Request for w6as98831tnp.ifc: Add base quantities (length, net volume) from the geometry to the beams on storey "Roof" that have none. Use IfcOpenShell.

First a look at what the model holds.

```python
import ifcopenshell
import ifcopenshell.util.element
import ifcopenshell.util.unit

model = ifcopenshell.open("w6as98831tnp.ifc")
print(model.schema)
for unit_type in ("LENGTHUNIT", "AREAUNIT", "VOLUMEUNIT"):
    print(unit_type, ifcopenshell.util.unit.calculate_unit_scale(model, unit_type))
storey = next(s for s in model.by_type("IfcBuildingStorey") if s.Name == "Roof")
beams = [e for e in ifcopenshell.util.element.get_decomposition(storey) if e.is_a("IfcBeam")]
for e in sorted(beams, key=lambda e: e.id()):
    print(e.id(), e.is_a(), e.Name, list(ifcopenshell.util.element.get_psets(e, qtos_only=True)), sep=" | ")
```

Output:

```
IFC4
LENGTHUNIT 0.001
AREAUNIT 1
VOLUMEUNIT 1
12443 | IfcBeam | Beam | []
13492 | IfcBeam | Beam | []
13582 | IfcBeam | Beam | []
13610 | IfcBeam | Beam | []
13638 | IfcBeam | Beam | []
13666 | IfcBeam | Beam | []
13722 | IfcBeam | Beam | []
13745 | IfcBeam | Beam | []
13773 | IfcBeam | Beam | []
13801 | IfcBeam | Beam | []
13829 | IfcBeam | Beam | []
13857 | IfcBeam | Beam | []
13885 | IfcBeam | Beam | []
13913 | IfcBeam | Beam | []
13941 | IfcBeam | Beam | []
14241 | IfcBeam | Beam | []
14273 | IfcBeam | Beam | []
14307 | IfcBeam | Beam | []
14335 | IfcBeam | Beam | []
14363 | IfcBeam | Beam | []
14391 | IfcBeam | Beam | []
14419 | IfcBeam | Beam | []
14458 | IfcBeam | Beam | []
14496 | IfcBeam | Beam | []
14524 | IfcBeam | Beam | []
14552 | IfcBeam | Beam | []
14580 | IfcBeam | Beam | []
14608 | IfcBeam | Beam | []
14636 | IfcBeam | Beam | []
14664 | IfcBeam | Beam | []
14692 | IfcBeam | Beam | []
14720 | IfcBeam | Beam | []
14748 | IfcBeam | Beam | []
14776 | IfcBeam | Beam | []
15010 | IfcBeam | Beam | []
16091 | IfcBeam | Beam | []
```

```python
import ifcopenshell
import ifcopenshell.api.pset
import ifcopenshell.geom
import ifcopenshell.util.element
import ifcopenshell.util.shape
import ifcopenshell.util.unit

model = ifcopenshell.open("w6as98831tnp.ifc")
unit_scale = ifcopenshell.util.unit.calculate_unit_scale(model)
volume_scale = ifcopenshell.util.unit.calculate_unit_scale(model, "VOLUMEUNIT")
settings = ifcopenshell.geom.settings()

storey = next(s for s in model.by_type("IfcBuildingStorey") if s.Name == "Roof")
beams = [e for e in ifcopenshell.util.element.get_decomposition(storey) if e.is_a("IfcBeam")]

for e in sorted(beams, key=lambda e: e.id()):
    if ifcopenshell.util.element.get_psets(e, qtos_only=True, should_inherit=False):
        continue
    # Geometry comes back in metres, in the element's own axes.
    shape = ifcopenshell.geom.create_shape(settings, e)
    values = {
        "Length": ifcopenshell.util.shape.get_max_xyz(shape.geometry) / unit_scale,
        "NetVolume": ifcopenshell.util.shape.get_volume(shape.geometry) / volume_scale,
    }
    qto = ifcopenshell.api.pset.add_qto(model, product=e, name="Qto_BeamBaseQuantities")
    ifcopenshell.api.pset.edit_qto(model, qto=qto, properties=values)
    print(e.id(), {k: round(v, 3) for k, v in values.items()})

model.write("w6as98831tnp_v2.ifc")
```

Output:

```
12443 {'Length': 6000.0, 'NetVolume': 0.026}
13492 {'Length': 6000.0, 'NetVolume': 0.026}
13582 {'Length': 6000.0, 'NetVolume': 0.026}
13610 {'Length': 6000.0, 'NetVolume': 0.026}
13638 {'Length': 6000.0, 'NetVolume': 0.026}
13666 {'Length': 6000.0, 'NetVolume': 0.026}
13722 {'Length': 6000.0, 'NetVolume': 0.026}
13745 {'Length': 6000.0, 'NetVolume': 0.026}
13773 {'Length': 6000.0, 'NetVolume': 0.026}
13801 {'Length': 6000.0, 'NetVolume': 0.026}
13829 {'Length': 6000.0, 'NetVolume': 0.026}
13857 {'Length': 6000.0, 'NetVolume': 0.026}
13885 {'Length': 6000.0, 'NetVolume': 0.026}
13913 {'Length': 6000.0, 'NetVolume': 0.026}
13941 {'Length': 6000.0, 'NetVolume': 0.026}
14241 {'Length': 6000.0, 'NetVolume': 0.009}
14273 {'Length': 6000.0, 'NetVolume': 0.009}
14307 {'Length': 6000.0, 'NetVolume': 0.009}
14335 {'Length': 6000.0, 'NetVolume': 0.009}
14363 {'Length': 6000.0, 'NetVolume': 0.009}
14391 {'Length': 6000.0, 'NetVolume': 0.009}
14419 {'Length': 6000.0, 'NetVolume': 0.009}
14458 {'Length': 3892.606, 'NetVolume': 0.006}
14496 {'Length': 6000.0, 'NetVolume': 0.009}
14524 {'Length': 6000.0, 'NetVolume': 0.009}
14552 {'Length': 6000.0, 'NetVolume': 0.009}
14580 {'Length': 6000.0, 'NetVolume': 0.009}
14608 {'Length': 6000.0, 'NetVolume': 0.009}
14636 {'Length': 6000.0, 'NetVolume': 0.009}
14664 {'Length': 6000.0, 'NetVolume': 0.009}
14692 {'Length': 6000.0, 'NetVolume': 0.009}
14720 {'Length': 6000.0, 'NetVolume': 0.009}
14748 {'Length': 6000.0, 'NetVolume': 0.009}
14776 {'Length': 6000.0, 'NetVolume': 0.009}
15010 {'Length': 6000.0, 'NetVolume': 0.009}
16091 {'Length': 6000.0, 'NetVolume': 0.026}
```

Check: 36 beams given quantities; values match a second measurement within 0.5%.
